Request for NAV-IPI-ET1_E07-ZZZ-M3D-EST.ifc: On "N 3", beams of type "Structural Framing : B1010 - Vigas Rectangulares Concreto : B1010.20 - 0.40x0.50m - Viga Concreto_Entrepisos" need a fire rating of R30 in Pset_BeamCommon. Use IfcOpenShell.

First a look at what the model holds.

```python
import ifcopenshell
import ifcopenshell.util.element

model = ifcopenshell.open("NAV-IPI-ET1_E07-ZZZ-M3D-EST.ifc")
print(model.schema)
storey = next(s for s in model.by_type("IfcBuildingStorey") if s.Name == "N 3")
beams = [e for e in ifcopenshell.util.element.get_decomposition(storey) if e.is_a("IfcBeam")]
seen = {}
for e in beams:
    element_type = ifcopenshell.util.element.get_type(e)
    key = (element_type.Name if element_type != e and element_type else None, ifcopenshell.util.element.get_pset(e, "Pset_BeamCommon", "FireRating"))
    seen[key] = seen.get(key, 0) + 1
for (name, value), count in sorted(seen.items(), key=str):
    print(count, "x", name, "|", value)
```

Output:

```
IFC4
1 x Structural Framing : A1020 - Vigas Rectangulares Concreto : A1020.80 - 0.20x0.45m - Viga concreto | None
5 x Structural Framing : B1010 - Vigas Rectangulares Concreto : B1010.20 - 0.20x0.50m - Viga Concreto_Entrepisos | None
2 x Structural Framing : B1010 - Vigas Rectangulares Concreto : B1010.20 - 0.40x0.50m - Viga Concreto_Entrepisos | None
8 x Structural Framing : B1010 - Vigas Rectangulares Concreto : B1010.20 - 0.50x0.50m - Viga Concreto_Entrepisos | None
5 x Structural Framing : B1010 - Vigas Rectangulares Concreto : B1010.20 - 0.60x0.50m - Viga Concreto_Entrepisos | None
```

```python
import ifcopenshell
import ifcopenshell.api.pset
import ifcopenshell.util.element

model = ifcopenshell.open("NAV-IPI-ET1_E07-ZZZ-M3D-EST.ifc")

storey = next(s for s in model.by_type("IfcBuildingStorey") if s.Name == "N 3")
beams = [e for e in ifcopenshell.util.element.get_decomposition(storey) if e.is_a("IfcBeam")]

count = 0
for e in beams:
    element_type = ifcopenshell.util.element.get_type(e)
    if element_type in (None, e) or element_type.Name != "Structural Framing : B1010 - Vigas Rectangulares Concreto : B1010.20 - 0.40x0.50m - Viga Concreto_Entrepisos":
        continue
    # add_pset returns the element's existing set when there is one.
    pset = ifcopenshell.api.pset.add_pset(model, product=e, name="Pset_BeamCommon")
    ifcopenshell.api.pset.edit_pset(model, pset=pset, properties={"FireRating": "R30"})
    count += 1

print(count, "beams updated")

model.write("NAV-IPI-ET1_E07-ZZZ-M3D-EST_updated.ifc")
```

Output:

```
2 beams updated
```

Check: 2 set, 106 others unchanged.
